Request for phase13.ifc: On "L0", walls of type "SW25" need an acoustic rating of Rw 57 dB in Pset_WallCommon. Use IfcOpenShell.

First a look at what the model holds.

```python
import ifcopenshell
import ifcopenshell.util.element

model = ifcopenshell.open("phase13.ifc")
print(model.schema)
storey = next(s for s in model.by_type("IfcBuildingStorey") if s.Name == "L0")
walls = [e for e in ifcopenshell.util.element.get_decomposition(storey) if e.is_a("IfcWall")]
seen = {}
for e in walls:
    element_type = ifcopenshell.util.element.get_type(e)
    key = (element_type.Name if element_type != e and element_type else None, ifcopenshell.util.element.get_pset(e, "Pset_WallCommon", "AcousticRating"))
    seen[key] = seen.get(key, 0) + 1
for (name, value), count in sorted(seen.items(), key=str):
    print(count, "x", name, "|", value)
```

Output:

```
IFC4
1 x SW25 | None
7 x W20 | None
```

```python
import ifcopenshell
import ifcopenshell.api.pset
import ifcopenshell.util.element

model = ifcopenshell.open("phase13.ifc")

storey = next(s for s in model.by_type("IfcBuildingStorey") if s.Name == "L0")
walls = [e for e in ifcopenshell.util.element.get_decomposition(storey) if e.is_a("IfcWall")]

count = 0
for e in walls:
    element_type = ifcopenshell.util.element.get_type(e)
    if element_type in (None, e) or element_type.Name != "SW25":
        continue
    # add_pset returns the element's existing set when there is one.
    pset = ifcopenshell.api.pset.add_pset(model, product=e, name="Pset_WallCommon")
    ifcopenshell.api.pset.edit_pset(model, pset=pset, properties={"AcousticRating": "Rw 57 dB"})
    count += 1

print(count, "walls updated")

model.write("phase13_edited.ifc")
```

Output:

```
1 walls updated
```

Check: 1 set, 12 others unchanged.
